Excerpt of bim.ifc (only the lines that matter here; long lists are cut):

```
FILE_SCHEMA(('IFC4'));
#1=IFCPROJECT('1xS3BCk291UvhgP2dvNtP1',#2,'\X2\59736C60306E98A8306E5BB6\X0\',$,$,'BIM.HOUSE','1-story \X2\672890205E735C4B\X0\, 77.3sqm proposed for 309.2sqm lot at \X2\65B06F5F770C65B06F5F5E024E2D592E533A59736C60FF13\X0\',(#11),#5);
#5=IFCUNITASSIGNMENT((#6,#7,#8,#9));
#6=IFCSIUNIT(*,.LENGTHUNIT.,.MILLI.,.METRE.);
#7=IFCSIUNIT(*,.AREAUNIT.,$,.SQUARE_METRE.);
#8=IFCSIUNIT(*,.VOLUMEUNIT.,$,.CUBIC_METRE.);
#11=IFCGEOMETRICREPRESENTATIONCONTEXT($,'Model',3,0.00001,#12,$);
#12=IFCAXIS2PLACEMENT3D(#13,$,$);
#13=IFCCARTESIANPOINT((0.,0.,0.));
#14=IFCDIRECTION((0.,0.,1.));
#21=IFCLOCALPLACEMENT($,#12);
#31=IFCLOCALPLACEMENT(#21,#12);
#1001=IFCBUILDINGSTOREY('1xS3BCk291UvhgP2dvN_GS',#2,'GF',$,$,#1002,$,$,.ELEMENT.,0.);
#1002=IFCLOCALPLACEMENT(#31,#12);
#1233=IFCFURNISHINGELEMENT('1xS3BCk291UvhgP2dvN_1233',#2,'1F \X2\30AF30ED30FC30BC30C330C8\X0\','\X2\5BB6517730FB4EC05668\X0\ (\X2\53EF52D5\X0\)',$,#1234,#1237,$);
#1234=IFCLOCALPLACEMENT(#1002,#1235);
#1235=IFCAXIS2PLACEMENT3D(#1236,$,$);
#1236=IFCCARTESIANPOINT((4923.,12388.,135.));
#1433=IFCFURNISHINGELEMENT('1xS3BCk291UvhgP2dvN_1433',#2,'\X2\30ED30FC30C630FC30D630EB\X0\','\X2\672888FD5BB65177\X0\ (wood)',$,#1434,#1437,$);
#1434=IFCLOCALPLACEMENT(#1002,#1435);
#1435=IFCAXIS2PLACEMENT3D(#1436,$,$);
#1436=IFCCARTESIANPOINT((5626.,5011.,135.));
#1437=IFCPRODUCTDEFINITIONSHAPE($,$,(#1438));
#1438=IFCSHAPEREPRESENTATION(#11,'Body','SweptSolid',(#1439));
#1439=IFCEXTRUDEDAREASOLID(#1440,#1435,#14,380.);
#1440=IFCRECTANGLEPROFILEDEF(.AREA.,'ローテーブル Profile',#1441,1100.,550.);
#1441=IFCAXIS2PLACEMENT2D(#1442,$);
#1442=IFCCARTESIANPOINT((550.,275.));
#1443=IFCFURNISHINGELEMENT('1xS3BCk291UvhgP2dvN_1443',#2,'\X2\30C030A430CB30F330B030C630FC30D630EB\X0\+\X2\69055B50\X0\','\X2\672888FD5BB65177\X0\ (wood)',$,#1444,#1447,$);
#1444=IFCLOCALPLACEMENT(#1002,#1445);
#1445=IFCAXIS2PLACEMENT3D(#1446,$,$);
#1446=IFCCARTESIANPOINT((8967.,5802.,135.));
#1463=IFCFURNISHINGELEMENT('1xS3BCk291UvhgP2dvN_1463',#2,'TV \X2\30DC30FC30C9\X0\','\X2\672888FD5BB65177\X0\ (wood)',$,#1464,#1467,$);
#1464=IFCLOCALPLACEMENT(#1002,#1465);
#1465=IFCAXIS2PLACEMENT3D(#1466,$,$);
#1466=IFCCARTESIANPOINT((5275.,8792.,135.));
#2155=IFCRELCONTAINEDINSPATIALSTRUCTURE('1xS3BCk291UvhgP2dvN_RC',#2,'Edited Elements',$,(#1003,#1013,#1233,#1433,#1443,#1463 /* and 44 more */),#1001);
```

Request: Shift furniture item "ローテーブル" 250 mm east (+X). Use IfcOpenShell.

```python
import ifcopenshell
import ifcopenshell.api.geometry
import ifcopenshell.util.placement
import ifcopenshell.util.unit

model = ifcopenshell.open("bim.ifc")
unit_scale = ifcopenshell.util.unit.calculate_unit_scale(model)

item = model.by_guid("1xS3BCk291UvhgP2dvN_1433")
matrix = ifcopenshell.util.placement.get_local_placement(item.ObjectPlacement)
matrix[0, 3] += 0.25 / unit_scale
ifcopenshell.api.geometry.edit_object_placement(model, product=item, matrix=matrix, is_si=False)

print(ifcopenshell.util.placement.get_local_placement(item.ObjectPlacement).round(3) + 0.0)

model.write("bim_updated.ifc")
```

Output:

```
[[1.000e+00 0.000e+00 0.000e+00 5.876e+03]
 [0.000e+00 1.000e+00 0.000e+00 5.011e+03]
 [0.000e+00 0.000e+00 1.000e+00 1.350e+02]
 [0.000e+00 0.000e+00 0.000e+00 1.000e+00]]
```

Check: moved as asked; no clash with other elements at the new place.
